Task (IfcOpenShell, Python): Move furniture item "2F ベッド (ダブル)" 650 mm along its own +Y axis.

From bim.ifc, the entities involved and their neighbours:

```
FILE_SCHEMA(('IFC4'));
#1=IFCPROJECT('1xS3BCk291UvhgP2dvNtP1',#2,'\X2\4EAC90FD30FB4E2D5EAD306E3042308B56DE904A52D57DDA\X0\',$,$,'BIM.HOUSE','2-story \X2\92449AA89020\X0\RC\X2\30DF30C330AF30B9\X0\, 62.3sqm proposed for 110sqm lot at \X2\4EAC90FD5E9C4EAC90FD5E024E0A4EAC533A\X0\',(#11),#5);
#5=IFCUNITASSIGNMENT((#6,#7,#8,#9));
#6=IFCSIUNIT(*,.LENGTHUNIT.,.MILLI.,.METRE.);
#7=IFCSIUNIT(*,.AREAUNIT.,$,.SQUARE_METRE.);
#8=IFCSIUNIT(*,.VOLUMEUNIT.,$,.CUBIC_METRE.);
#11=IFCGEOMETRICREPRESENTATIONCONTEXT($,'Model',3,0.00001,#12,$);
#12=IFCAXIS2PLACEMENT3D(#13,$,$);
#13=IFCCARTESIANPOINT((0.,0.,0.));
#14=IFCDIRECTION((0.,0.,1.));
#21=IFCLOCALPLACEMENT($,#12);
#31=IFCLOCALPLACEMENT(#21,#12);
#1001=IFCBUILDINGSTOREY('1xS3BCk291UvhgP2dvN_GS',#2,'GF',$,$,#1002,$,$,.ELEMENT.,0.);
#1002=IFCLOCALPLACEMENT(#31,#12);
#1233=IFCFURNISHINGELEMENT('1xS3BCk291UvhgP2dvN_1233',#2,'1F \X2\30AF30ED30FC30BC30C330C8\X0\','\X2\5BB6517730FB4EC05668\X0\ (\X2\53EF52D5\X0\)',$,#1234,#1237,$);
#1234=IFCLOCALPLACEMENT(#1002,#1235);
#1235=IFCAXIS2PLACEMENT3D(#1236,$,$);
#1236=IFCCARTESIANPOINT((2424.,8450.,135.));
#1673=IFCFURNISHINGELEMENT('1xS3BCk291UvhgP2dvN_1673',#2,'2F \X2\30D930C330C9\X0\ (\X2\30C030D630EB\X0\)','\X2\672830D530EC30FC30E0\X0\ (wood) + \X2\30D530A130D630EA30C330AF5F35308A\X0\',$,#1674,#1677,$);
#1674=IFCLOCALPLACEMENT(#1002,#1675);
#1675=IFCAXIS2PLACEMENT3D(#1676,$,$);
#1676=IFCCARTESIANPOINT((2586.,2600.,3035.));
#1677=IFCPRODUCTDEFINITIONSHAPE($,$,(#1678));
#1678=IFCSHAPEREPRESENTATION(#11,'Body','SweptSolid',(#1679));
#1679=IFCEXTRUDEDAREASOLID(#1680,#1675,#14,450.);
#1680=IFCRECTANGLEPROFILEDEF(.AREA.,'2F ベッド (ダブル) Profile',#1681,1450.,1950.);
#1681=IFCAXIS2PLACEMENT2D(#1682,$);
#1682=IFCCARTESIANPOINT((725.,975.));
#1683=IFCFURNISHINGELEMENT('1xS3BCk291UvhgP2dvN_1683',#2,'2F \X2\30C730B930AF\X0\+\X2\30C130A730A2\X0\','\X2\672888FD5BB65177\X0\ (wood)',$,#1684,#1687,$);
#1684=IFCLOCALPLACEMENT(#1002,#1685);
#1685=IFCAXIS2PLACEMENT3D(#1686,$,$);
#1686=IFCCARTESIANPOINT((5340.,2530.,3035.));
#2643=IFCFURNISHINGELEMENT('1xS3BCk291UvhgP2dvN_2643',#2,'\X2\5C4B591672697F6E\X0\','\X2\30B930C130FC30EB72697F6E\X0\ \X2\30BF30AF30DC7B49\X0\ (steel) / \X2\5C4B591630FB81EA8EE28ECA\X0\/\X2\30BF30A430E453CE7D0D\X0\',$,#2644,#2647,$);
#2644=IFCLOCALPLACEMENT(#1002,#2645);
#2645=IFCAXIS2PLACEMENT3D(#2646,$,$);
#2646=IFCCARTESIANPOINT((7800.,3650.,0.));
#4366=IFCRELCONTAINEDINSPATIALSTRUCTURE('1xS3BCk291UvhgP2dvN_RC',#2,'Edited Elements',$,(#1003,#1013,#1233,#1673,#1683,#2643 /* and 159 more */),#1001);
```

```python
import ifcopenshell
import ifcopenshell.api.geometry
import ifcopenshell.util.placement

model = ifcopenshell.open("bim.ifc")

item = model.by_guid("1xS3BCk291UvhgP2dvN_1673")
matrix = ifcopenshell.util.placement.get_local_placement(item.ObjectPlacement)
matrix[:3, 3] += matrix[:3, 1] * 650.0
ifcopenshell.api.geometry.edit_object_placement(model, product=item, matrix=matrix, is_si=False)

print(ifcopenshell.util.placement.get_local_placement(item.ObjectPlacement).round(3) + 0.0)

model.write("bim-out.ifc")
```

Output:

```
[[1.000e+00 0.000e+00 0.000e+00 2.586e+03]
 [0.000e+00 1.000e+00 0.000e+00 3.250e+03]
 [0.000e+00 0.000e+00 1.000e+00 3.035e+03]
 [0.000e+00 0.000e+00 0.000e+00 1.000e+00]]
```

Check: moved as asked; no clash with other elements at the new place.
